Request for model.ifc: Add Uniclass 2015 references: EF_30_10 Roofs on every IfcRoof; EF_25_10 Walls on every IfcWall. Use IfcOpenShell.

First a look at what the model holds.

```python
import ifcopenshell

model = ifcopenshell.open("model.ifc")
print(model.schema)
print("classifications:", [c.Name for c in model.by_type("IfcClassification")])
for ifc_class in ("IfcDoor", "IfcRoof", "IfcStair", "IfcWall", "IfcWindow"):
    print(ifc_class, len(model.by_type(ifc_class)))
```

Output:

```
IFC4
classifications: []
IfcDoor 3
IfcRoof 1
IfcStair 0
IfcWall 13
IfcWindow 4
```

```python
import ifcopenshell
import ifcopenshell.api.classification

model = ifcopenshell.open("model.ifc")

system = ifcopenshell.api.classification.add_classification(model, classification="Uniclass 2015")

codes = {
    "IfcRoof": ("EF_30_10", "Roofs"),
    "IfcWall": ("EF_25_10", "Walls"),
}
for ifc_class, (code, name) in codes.items():
    products = model.by_type(ifc_class)
    ifcopenshell.api.classification.add_reference(
        model, products=products, classification=system, identification=code, name=name
    )
    print(code, len(products))

model.write("model-out.ifc")
```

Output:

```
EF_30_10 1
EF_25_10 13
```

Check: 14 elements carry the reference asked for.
